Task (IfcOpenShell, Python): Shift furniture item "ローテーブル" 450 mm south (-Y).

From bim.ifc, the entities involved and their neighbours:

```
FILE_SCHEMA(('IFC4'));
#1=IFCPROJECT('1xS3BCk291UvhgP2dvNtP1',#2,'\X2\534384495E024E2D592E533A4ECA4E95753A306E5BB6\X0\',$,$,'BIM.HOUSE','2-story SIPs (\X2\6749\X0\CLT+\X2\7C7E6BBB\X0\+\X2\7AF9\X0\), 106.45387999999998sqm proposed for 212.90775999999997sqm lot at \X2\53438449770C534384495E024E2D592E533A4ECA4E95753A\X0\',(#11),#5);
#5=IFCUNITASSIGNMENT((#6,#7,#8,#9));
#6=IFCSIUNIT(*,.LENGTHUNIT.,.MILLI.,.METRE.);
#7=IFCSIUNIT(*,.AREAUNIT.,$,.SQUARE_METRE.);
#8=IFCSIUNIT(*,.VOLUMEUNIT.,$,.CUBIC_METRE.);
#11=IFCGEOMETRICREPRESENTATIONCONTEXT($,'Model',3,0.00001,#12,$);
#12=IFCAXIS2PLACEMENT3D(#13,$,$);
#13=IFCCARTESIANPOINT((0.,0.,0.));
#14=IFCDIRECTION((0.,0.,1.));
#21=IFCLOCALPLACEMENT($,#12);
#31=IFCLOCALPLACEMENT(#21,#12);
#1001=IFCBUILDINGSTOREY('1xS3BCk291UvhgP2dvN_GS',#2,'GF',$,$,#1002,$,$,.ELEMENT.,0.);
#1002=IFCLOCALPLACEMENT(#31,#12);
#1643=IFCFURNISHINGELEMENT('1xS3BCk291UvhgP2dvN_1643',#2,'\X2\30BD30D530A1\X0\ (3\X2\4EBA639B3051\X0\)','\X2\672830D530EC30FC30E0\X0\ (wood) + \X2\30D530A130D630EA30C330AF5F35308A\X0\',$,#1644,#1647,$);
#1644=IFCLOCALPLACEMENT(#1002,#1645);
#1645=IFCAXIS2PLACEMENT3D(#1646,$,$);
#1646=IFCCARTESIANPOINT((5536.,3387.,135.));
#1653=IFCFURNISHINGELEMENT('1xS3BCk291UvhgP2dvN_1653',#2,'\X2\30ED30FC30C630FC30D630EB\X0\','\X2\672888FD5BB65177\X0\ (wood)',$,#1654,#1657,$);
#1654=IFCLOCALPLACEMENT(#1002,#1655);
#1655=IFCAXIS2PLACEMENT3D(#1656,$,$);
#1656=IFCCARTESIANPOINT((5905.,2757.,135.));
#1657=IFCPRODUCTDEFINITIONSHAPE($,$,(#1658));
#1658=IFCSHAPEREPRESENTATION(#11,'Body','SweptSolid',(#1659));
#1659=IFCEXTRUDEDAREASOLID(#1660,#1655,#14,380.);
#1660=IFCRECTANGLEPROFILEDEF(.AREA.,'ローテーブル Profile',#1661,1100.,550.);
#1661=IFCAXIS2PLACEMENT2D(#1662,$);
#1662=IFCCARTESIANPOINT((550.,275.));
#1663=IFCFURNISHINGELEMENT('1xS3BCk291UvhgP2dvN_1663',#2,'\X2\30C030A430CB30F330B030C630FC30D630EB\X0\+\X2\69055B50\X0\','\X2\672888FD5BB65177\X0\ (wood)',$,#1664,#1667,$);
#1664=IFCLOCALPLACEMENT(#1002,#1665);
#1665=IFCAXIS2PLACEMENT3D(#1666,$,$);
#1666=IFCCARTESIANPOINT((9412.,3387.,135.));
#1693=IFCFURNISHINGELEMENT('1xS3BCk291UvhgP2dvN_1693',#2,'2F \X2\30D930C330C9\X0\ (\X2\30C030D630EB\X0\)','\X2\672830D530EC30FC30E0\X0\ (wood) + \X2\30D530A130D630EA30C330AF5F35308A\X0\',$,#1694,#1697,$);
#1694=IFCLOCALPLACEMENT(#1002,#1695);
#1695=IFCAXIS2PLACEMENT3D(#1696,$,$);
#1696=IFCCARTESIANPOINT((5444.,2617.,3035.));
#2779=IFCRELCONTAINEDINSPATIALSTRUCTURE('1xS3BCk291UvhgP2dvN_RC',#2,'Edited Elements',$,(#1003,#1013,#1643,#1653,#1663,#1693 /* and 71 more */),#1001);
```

```python
import ifcopenshell
import ifcopenshell.api.geometry
import ifcopenshell.util.placement
import ifcopenshell.util.unit

model = ifcopenshell.open("bim.ifc")
unit_scale = ifcopenshell.util.unit.calculate_unit_scale(model)

item = model.by_guid("1xS3BCk291UvhgP2dvN_1653")
matrix = ifcopenshell.util.placement.get_local_placement(item.ObjectPlacement)
matrix[1, 3] -= 0.45 / unit_scale
ifcopenshell.api.geometry.edit_object_placement(model, product=item, matrix=matrix, is_si=False)

print(ifcopenshell.util.placement.get_local_placement(item.ObjectPlacement).round(3) + 0.0)

model.write("bim_edited.ifc")
```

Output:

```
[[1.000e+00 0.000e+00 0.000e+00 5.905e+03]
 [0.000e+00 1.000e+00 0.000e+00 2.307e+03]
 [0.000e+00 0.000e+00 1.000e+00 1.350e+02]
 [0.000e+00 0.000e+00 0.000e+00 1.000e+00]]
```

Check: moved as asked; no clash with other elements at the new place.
